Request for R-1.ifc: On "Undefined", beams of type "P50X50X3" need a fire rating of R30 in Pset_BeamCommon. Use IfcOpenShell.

First a look at what the model holds.

```python
import ifcopenshell
import ifcopenshell.util.element

model = ifcopenshell.open("R-1.ifc")
print(model.schema)
storey = next(s for s in model.by_type("IfcBuildingStorey") if s.Name == "Undefined")
beams = [e for e in ifcopenshell.util.element.get_decomposition(storey) if e.is_a("IfcBeam")]
seen = {}
for e in beams:
    element_type = ifcopenshell.util.element.get_type(e)
    key = (element_type.Name if element_type != e and element_type else None, ifcopenshell.util.element.get_pset(e, "Pset_BeamCommon", "FireRating"))
    seen[key] = seen.get(key, 0) + 1
for (name, value), count in sorted(seen.items(), key=str):
    print(count, "x", name, "|", value)
```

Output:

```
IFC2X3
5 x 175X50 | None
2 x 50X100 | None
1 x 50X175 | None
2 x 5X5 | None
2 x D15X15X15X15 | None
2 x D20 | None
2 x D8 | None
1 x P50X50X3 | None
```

```python
import ifcopenshell
import ifcopenshell.api.pset
import ifcopenshell.util.element

model = ifcopenshell.open("R-1.ifc")

storey = next(s for s in model.by_type("IfcBuildingStorey") if s.Name == "Undefined")
beams = [e for e in ifcopenshell.util.element.get_decomposition(storey) if e.is_a("IfcBeam")]

count = 0
for e in beams:
    element_type = ifcopenshell.util.element.get_type(e)
    if element_type in (None, e) or element_type.Name != "P50X50X3":
        continue
    # add_pset returns the element's existing set when there is one.
    pset = ifcopenshell.api.pset.add_pset(model, product=e, name="Pset_BeamCommon")
    ifcopenshell.api.pset.edit_pset(model, pset=pset, properties={"FireRating": "R30"})
    count += 1

print(count, "beams updated")

model.write("R-1_edited.ifc")
```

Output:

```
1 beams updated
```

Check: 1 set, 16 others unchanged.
